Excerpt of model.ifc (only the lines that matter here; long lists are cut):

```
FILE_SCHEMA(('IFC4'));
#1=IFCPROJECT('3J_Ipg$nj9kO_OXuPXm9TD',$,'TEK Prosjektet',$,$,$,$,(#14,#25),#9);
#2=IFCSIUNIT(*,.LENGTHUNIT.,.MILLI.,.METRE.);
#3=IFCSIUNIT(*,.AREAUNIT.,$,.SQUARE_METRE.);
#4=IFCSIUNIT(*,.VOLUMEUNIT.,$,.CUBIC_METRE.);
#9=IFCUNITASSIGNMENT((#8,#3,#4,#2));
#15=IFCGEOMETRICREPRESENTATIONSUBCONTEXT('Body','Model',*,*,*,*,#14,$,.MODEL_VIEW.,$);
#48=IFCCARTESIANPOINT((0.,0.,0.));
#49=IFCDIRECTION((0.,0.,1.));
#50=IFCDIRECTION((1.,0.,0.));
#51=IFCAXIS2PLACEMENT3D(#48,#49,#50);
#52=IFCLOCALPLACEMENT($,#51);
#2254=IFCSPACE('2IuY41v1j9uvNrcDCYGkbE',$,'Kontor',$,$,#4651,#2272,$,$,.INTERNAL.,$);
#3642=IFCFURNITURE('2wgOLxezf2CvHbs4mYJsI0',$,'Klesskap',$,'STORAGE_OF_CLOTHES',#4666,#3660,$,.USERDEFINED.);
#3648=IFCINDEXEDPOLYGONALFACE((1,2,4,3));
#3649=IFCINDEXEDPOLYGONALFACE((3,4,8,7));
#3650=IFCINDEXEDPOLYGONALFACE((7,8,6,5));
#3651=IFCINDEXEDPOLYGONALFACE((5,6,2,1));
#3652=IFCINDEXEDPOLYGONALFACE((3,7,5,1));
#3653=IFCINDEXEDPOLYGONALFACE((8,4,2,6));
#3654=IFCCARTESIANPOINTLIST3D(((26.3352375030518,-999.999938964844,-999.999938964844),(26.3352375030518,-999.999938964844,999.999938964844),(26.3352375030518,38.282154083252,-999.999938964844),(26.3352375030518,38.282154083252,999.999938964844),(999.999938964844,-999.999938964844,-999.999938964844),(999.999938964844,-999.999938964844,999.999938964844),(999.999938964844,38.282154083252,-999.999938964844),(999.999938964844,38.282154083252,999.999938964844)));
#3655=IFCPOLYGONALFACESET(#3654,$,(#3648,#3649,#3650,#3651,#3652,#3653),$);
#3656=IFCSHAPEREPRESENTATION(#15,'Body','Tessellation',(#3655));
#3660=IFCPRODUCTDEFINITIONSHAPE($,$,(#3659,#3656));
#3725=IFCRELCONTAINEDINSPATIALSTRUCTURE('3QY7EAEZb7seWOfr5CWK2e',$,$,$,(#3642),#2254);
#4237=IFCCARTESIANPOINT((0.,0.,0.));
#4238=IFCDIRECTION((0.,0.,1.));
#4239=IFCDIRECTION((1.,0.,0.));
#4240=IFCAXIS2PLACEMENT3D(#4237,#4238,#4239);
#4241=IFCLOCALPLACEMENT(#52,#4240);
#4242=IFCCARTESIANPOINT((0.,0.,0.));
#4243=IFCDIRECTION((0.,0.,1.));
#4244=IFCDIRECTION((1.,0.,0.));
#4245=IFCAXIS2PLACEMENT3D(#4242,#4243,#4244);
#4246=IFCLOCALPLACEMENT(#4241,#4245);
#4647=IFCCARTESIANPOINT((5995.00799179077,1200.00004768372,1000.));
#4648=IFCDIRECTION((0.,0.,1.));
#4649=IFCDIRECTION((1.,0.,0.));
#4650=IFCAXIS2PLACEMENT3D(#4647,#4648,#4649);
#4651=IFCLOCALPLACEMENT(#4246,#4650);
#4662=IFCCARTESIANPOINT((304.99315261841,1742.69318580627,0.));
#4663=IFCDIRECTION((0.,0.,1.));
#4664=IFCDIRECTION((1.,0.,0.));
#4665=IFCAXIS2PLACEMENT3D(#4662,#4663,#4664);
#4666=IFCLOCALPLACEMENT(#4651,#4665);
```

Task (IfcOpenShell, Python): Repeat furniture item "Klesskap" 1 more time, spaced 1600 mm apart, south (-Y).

```python
import numpy as np
import ifcopenshell
import ifcopenshell.api.geometry
import ifcopenshell.api.root
import ifcopenshell.util.element
import ifcopenshell.util.placement
import ifcopenshell.util.unit

model = ifcopenshell.open("model.ifc")
unit_scale = ifcopenshell.util.unit.calculate_unit_scale(model)

source = model.by_guid("2wgOLxezf2CvHbs4mYJsI0")
base = ifcopenshell.util.placement.get_local_placement(source.ObjectPlacement)
step = np.array([0.0, -1.0, 0.0]) * 1.6 / unit_scale

for i in range(1, 2):
    copy = ifcopenshell.api.root.copy_class(model, product=source)
    copy.Representation = ifcopenshell.util.element.copy_deep(
        model, source.Representation, exclude=["IfcGeometricRepresentationContext", "IfcRepresentationMap"]
    )
    matrix = base.copy()
    matrix[:3, 3] += i * step
    print("added at", matrix[:3, 3].round(3) + 0.0)
    ifcopenshell.api.geometry.edit_object_placement(model, product=copy, matrix=matrix, is_si=False)

model.write("model_v2.ifc")
```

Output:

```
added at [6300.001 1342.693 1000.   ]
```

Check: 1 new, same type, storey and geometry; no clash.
